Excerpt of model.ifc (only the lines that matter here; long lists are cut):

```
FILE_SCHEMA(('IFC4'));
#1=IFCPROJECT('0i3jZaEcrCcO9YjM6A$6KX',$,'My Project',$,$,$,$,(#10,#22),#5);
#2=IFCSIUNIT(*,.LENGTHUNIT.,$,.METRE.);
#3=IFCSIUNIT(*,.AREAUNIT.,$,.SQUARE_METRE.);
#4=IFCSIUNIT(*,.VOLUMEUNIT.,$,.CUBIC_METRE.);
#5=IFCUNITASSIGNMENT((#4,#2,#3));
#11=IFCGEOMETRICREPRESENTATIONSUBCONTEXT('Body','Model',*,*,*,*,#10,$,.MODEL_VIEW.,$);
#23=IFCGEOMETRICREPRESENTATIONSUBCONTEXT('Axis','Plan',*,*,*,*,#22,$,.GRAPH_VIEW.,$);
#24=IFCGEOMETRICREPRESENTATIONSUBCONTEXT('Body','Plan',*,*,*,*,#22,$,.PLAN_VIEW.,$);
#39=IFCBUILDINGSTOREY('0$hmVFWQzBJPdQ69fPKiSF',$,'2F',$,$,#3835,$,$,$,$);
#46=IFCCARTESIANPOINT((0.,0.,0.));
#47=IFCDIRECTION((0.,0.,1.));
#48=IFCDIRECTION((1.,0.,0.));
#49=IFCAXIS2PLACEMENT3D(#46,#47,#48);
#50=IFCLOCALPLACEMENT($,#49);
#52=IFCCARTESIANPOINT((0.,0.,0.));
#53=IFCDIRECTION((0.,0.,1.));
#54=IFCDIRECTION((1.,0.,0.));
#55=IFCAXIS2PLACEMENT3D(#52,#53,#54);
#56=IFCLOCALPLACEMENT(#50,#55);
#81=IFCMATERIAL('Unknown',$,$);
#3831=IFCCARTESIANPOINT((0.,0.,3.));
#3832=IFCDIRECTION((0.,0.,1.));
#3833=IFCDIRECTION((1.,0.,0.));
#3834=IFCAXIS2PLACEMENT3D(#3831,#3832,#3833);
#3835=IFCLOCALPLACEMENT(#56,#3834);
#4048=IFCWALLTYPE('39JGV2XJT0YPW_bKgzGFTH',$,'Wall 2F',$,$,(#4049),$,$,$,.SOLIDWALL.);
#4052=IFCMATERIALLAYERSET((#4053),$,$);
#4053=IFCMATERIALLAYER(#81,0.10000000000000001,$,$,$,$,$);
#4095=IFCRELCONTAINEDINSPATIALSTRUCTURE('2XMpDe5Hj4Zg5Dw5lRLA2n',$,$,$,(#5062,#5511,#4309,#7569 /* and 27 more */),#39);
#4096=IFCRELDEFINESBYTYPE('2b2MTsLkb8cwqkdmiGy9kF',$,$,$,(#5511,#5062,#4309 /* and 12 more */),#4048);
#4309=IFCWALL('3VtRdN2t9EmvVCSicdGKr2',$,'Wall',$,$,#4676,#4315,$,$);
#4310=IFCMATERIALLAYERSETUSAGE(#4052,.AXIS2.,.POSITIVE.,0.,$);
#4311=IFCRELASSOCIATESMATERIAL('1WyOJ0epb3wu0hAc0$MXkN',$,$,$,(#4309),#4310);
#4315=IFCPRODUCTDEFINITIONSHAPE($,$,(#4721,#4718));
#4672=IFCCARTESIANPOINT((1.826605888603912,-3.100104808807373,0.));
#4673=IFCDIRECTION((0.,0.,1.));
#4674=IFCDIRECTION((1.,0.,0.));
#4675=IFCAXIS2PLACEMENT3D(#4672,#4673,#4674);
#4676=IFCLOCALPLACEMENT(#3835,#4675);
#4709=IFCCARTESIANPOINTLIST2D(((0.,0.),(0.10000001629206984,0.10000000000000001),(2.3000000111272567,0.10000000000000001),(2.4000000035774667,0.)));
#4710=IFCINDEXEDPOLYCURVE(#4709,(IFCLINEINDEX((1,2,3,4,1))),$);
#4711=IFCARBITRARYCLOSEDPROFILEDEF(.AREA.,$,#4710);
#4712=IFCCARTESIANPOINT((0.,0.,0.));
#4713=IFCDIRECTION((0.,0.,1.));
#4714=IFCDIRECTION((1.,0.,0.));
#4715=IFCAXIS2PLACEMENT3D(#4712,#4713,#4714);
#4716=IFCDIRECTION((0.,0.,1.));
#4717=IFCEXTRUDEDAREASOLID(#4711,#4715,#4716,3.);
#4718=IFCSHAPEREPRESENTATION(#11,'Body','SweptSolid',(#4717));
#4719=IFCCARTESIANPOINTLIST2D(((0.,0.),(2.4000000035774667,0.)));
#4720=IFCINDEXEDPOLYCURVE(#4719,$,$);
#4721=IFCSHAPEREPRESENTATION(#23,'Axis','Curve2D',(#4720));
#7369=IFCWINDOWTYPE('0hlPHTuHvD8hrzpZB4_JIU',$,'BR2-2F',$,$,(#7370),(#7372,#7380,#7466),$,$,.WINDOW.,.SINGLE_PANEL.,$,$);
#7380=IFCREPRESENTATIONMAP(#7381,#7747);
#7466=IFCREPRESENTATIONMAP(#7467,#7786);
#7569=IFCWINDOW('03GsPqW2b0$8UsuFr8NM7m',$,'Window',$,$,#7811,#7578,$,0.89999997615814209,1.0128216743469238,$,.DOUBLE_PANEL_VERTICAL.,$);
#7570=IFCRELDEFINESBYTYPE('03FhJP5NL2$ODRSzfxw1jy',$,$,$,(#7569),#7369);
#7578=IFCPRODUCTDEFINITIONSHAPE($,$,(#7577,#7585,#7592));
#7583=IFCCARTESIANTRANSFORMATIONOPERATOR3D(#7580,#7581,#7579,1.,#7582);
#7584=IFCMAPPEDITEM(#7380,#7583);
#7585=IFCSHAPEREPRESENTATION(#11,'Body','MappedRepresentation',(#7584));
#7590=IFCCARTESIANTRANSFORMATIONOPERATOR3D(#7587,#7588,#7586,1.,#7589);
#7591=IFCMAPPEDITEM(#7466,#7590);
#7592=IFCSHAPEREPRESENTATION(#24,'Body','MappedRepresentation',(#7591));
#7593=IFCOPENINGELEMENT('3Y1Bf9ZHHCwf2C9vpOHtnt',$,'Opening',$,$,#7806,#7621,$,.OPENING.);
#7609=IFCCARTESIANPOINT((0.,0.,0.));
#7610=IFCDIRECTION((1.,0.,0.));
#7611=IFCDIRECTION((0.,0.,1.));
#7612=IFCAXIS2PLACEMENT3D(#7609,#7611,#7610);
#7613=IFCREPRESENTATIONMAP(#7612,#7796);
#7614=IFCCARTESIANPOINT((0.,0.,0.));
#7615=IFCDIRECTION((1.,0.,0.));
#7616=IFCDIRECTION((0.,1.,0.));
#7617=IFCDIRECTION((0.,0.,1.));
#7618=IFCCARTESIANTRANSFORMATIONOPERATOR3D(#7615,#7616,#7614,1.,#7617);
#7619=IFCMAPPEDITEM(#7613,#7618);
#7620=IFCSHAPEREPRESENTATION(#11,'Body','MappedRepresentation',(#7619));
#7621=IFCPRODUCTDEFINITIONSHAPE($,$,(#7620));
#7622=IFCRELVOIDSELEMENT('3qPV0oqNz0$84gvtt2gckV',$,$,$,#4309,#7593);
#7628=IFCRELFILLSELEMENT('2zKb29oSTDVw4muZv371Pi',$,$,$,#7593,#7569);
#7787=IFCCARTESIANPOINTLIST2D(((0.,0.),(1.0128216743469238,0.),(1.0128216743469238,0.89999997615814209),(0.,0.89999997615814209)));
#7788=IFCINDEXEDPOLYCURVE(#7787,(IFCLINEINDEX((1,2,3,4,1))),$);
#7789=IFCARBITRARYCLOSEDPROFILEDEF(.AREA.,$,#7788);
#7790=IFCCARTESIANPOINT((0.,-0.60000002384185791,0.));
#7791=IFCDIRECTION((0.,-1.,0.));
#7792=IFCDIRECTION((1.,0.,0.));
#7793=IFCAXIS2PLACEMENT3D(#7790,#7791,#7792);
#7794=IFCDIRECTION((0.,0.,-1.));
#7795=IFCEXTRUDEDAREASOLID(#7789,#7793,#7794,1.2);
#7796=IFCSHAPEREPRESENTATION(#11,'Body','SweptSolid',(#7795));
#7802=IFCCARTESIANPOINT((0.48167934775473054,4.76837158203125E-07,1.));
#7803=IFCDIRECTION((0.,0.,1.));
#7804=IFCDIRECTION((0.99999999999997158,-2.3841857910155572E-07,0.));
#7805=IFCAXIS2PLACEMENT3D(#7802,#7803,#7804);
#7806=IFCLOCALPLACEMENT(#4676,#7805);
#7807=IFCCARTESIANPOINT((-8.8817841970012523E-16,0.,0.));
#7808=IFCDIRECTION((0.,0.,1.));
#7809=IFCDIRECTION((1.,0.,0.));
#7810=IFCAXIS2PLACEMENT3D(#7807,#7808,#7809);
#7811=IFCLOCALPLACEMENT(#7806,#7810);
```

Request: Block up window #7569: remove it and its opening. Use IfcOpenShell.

```python
import ifcopenshell
import ifcopenshell.api.feature
import ifcopenshell.api.root
import ifcopenshell.geom
import ifcopenshell.util.shape

model = ifcopenshell.open("model.ifc")
settings = ifcopenshell.geom.settings()


def volume(element):
    """Net volume in cubic metres, openings subtracted."""
    shape = ifcopenshell.geom.create_shape(settings, element)
    return ifcopenshell.util.shape.get_volume(shape.geometry)


window = model.by_id(7569)
opening = window.FillsVoids[0].RelatingOpeningElement
wall = opening.VoidsElements[0].RelatingBuildingElement
before = volume(wall)

ifcopenshell.api.root.remove_product(model, product=window)
ifcopenshell.api.feature.remove_feature(model, feature=opening)

after = volume(wall)

print(f"wall volume {before:.3f} -> {after:.3f} m3")

model.write("model-out.ifc")
```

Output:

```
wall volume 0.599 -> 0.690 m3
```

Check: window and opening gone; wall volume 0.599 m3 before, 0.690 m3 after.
